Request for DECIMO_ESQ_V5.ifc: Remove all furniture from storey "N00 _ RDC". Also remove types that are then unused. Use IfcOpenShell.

First a look at what the model holds.

```python
import ifcopenshell
import ifcopenshell.util.element

model = ifcopenshell.open("DECIMO_ESQ_V5.ifc")
print(model.schema)
storey = next(s for s in model.by_type("IfcBuildingStorey") if s.Name == "N00 _ RDC")
furniture = [e for e in ifcopenshell.util.element.get_decomposition(storey) if e.is_a("IfcFurnishingElement")]
seen = {}
for e in furniture:
    element_type = ifcopenshell.util.element.get_type(e)
    name = element_type.Name if element_type not in (None, e) else None
    seen[name] = seen.get(name, 0) + 1
for name, count in sorted(seen.items(), key=str):
    print(count, "x", name)
```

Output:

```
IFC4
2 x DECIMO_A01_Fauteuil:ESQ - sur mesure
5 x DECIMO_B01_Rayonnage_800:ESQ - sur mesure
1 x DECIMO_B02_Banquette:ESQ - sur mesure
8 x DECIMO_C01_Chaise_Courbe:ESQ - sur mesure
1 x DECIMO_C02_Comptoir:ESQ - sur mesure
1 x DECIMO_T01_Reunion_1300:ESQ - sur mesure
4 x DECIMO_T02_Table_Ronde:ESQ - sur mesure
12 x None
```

```python
import ifcopenshell
import ifcopenshell.api.root
import ifcopenshell.util.element

model = ifcopenshell.open("DECIMO_ESQ_V5.ifc")

storey = next(s for s in model.by_type("IfcBuildingStorey") if s.Name == "N00 _ RDC")
furniture = [e for e in ifcopenshell.util.element.get_decomposition(storey) if e.is_a("IfcFurnishingElement")]
types = {ifcopenshell.util.element.get_type(e) for e in furniture} - {None, *furniture}

for e in furniture:
    ifcopenshell.api.root.remove_product(model, product=e)
print(len(furniture), "removed")

unused = [t for t in types if not ifcopenshell.util.element.get_types(t)]
for t in unused:
    ifcopenshell.api.root.remove_product(model, product=t)
print(len(unused), "unused types removed")

model.write("DECIMO_ESQ_V5_updated.ifc")
```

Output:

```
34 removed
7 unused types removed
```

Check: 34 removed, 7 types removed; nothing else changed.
